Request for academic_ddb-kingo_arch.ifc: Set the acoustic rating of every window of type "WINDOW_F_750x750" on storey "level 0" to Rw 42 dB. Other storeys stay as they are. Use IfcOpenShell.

First a look at what the model holds.

```python
import ifcopenshell
import ifcopenshell.util.element

model = ifcopenshell.open("academic_ddb-kingo_arch.ifc")
print(model.schema)
storey = next(s for s in model.by_type("IfcBuildingStorey") if s.Name == "level 0")
windows = [e for e in ifcopenshell.util.element.get_decomposition(storey) if e.is_a("IfcWindow")]
seen = {}
for e in windows:
    element_type = ifcopenshell.util.element.get_type(e)
    key = (element_type.Name if element_type != e and element_type else None, ifcopenshell.util.element.get_pset(e, "Pset_WindowCommon", "AcousticRating"))
    seen[key] = seen.get(key, 0) + 1
for (name, value), count in sorted(seen.items(), key=str):
    print(count, "x", name, "|", value)
```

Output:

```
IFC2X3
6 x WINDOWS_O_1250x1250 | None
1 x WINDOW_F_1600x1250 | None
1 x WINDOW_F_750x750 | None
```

```python
import ifcopenshell
import ifcopenshell.api.pset
import ifcopenshell.util.element

model = ifcopenshell.open("academic_ddb-kingo_arch.ifc")

storey = next(s for s in model.by_type("IfcBuildingStorey") if s.Name == "level 0")
windows = [e for e in ifcopenshell.util.element.get_decomposition(storey) if e.is_a("IfcWindow")]

count = 0
for e in windows:
    element_type = ifcopenshell.util.element.get_type(e)
    if element_type in (None, e) or element_type.Name != "WINDOW_F_750x750":
        continue
    # add_pset returns the element's existing set when there is one.
    pset = ifcopenshell.api.pset.add_pset(model, product=e, name="Pset_WindowCommon")
    ifcopenshell.api.pset.edit_pset(model, pset=pset, properties={"AcousticRating": "Rw 42 dB"})
    count += 1

print(count, "windows updated")

model.write("academic_ddb-kingo_arch_edited.ifc")
```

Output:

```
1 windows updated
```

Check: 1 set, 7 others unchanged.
